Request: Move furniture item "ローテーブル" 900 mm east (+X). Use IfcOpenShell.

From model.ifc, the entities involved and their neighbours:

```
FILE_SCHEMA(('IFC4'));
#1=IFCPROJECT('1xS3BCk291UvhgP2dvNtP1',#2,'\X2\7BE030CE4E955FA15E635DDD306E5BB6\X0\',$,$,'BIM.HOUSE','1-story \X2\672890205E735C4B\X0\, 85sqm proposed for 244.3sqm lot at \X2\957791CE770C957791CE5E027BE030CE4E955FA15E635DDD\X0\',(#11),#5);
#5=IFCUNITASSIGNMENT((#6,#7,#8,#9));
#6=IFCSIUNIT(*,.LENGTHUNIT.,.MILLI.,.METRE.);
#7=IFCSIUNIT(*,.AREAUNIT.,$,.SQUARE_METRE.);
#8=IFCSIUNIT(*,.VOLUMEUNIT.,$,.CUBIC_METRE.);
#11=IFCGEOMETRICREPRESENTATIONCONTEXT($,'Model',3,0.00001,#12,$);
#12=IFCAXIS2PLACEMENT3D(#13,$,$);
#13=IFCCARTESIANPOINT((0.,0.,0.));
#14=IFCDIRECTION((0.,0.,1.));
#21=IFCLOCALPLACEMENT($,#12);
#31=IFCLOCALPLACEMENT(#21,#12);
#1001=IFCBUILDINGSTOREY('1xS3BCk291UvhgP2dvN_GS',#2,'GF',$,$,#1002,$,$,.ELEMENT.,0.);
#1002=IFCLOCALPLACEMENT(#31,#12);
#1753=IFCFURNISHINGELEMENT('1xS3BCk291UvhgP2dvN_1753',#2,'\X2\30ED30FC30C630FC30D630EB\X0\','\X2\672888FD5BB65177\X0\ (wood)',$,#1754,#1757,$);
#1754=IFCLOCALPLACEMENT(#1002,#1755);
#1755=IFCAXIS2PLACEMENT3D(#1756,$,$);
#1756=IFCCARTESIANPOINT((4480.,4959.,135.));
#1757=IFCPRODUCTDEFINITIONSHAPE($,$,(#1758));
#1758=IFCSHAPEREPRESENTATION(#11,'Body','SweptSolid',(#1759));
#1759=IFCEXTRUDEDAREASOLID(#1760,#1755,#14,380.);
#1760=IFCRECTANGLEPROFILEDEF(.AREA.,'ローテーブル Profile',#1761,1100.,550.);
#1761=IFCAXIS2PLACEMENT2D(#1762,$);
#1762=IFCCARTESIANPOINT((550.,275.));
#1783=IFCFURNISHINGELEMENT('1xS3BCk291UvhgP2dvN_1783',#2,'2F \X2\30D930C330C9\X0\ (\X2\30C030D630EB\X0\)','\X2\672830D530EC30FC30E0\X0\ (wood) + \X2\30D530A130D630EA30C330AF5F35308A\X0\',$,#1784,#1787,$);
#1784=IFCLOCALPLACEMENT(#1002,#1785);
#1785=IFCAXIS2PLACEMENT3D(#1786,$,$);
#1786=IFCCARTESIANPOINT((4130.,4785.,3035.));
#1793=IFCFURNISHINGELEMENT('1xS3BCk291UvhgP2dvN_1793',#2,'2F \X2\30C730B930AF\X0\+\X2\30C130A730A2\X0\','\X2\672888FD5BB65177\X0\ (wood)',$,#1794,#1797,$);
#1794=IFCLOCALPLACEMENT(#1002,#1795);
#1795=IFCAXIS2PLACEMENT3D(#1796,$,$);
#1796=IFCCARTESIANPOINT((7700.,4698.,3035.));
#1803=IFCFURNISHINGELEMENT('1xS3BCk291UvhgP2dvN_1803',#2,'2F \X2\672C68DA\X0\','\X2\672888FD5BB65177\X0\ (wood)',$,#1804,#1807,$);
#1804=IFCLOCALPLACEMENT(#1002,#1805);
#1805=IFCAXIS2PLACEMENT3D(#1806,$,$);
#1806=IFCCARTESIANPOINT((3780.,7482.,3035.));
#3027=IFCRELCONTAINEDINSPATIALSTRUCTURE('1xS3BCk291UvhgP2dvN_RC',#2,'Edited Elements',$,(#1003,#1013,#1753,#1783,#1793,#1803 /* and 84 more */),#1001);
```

```python
import ifcopenshell
import ifcopenshell.api.geometry
import ifcopenshell.util.placement
import ifcopenshell.util.unit

model = ifcopenshell.open("model.ifc")
unit_scale = ifcopenshell.util.unit.calculate_unit_scale(model)

item = model.by_id(1753)
matrix = ifcopenshell.util.placement.get_local_placement(item.ObjectPlacement)
matrix[0, 3] += 0.9 / unit_scale
ifcopenshell.api.geometry.edit_object_placement(model, product=item, matrix=matrix, is_si=False)

print(ifcopenshell.util.placement.get_local_placement(item.ObjectPlacement).round(3) + 0.0)

model.write("model_updated.ifc")
```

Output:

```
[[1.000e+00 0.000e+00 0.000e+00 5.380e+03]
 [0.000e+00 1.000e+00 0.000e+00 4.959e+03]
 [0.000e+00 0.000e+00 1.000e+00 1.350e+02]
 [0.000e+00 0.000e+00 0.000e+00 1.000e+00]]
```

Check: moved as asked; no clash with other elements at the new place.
